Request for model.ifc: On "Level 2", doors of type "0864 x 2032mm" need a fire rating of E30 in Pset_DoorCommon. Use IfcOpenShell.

First a look at what the model holds.

```python
import ifcopenshell
import ifcopenshell.util.element

model = ifcopenshell.open("model.ifc")
print(model.schema)
storey = next(s for s in model.by_type("IfcBuildingStorey") if s.Name == "Level 2")
doors = [e for e in ifcopenshell.util.element.get_decomposition(storey) if e.is_a("IfcDoor")]
seen = {}
for e in doors:
    element_type = ifcopenshell.util.element.get_type(e)
    key = (element_type.Name if element_type != e and element_type else None, ifcopenshell.util.element.get_pset(e, "Pset_DoorCommon", "FireRating"))
    seen[key] = seen.get(key, 0) + 1
for (name, value), count in sorted(seen.items(), key=str):
    print(count, "x", name, "|", value)
```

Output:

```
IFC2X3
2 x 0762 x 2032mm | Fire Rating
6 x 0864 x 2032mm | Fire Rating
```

```python
import ifcopenshell
import ifcopenshell.api.pset
import ifcopenshell.util.element

model = ifcopenshell.open("model.ifc")

storey = next(s for s in model.by_type("IfcBuildingStorey") if s.Name == "Level 2")
doors = [e for e in ifcopenshell.util.element.get_decomposition(storey) if e.is_a("IfcDoor")]

count = 0
for e in doors:
    element_type = ifcopenshell.util.element.get_type(e)
    if element_type in (None, e) or element_type.Name != "0864 x 2032mm":
        continue
    # add_pset returns the element's existing set when there is one.
    pset = ifcopenshell.api.pset.add_pset(model, product=e, name="Pset_DoorCommon")
    ifcopenshell.api.pset.edit_pset(model, pset=pset, properties={"FireRating": "E30"})
    count += 1

print(count, "doors updated")

model.write("model_v2.ifc")
```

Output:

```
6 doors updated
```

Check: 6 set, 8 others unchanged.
